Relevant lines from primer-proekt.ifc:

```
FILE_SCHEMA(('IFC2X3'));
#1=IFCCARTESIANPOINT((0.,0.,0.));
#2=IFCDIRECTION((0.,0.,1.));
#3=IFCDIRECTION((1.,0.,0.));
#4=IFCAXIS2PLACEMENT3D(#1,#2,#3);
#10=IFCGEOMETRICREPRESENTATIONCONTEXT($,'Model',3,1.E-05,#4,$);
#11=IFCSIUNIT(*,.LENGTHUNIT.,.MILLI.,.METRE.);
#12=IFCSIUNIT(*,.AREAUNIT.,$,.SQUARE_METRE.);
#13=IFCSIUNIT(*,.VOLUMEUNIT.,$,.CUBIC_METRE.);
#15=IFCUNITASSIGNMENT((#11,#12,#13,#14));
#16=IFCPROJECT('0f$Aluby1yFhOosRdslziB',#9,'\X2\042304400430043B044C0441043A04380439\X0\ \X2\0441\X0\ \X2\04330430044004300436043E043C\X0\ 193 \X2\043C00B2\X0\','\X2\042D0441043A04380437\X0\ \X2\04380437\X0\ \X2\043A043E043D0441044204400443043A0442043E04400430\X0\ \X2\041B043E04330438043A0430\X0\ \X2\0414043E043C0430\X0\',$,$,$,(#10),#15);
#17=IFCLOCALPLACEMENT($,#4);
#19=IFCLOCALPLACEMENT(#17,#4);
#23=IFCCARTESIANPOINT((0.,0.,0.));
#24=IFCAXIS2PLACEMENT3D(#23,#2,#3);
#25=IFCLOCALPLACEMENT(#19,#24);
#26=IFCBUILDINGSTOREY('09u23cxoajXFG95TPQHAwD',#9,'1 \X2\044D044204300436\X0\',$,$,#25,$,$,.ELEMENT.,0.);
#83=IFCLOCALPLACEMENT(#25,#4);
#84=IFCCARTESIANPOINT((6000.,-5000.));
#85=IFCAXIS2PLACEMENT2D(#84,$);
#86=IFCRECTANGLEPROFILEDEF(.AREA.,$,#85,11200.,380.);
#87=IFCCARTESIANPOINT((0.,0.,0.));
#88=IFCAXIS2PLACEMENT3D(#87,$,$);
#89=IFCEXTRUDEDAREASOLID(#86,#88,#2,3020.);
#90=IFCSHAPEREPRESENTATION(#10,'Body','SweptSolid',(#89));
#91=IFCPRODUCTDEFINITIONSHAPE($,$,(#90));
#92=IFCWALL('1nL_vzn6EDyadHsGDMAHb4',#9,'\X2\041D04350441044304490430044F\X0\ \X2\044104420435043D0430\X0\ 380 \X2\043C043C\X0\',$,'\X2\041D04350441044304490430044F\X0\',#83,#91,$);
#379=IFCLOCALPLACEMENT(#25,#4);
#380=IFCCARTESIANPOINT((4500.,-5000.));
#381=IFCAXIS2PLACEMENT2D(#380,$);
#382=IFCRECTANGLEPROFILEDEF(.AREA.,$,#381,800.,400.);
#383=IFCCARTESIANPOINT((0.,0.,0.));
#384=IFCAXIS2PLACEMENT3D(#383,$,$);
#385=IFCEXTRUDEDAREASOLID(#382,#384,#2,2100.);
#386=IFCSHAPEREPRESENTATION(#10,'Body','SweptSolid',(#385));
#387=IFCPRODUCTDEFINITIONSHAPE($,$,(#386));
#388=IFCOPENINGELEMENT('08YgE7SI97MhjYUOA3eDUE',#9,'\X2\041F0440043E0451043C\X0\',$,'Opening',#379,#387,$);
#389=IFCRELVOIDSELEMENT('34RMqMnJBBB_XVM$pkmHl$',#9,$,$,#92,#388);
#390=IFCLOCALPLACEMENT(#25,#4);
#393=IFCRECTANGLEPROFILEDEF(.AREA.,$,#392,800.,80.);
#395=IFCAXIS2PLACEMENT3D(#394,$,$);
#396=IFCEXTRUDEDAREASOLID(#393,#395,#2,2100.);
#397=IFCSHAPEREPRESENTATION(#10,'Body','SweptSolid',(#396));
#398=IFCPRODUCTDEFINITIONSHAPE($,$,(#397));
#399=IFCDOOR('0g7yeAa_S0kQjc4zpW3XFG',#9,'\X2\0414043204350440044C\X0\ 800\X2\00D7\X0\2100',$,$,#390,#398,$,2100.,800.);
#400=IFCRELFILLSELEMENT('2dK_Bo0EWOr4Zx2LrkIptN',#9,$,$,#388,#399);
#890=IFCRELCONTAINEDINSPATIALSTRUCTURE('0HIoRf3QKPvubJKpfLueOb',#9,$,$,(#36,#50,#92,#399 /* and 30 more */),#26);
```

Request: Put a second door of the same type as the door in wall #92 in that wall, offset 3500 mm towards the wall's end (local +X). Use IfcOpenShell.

```python
import ifcopenshell
import ifcopenshell.api.feature
import ifcopenshell.api.geometry
import ifcopenshell.api.root
import ifcopenshell.geom
import ifcopenshell.util.element
import ifcopenshell.util.placement
import ifcopenshell.util.shape
import ifcopenshell.util.unit

model = ifcopenshell.open("primer-proekt.ifc")
unit_scale = ifcopenshell.util.unit.calculate_unit_scale(model)
settings = ifcopenshell.geom.settings()


def volume(element):
    """Net volume in cubic metres, openings subtracted."""
    shape = ifcopenshell.geom.create_shape(settings, element)
    return ifcopenshell.util.shape.get_volume(shape.geometry)


door = model.by_id(399)
opening = door.FillsVoids[0].RelatingOpeningElement
wall = opening.VoidsElements[0].RelatingBuildingElement
before = volume(wall)
shift = ifcopenshell.util.placement.get_local_placement(wall.ObjectPlacement)[:3, 0] * 3.5 / unit_scale

# copy_class copies the void relationship, type, container and properties, but no geometry.
new_opening = ifcopenshell.api.root.copy_class(model, product=opening)
new_opening.Representation = ifcopenshell.util.element.copy_deep(
    model, opening.Representation, exclude=["IfcGeometricRepresentationContext", "IfcRepresentationMap"]
)
new_door = ifcopenshell.api.root.copy_class(model, product=door)
new_door.Representation = ifcopenshell.util.element.copy_deep(
    model, door.Representation, exclude=["IfcGeometricRepresentationContext", "IfcRepresentationMap"]
)
fills = ifcopenshell.api.feature.add_filling(model, opening=new_opening, element=new_door)
fills.OwnerHistory = new_door.OwnerHistory  # required in IFC2X3

for old, new in ((opening, new_opening), (door, new_door)):
    matrix = ifcopenshell.util.placement.get_local_placement(old.ObjectPlacement)
    matrix[:3, 3] += shift
    ifcopenshell.api.geometry.edit_object_placement(model, product=new, matrix=matrix, is_si=False)

after = volume(wall)

print(f"wall volume {before:.3f} -> {after:.3f} m3")

model.write("primer-proekt_updated.ifc")
```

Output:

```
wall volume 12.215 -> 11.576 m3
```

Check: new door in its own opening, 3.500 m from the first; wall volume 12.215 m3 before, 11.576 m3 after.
